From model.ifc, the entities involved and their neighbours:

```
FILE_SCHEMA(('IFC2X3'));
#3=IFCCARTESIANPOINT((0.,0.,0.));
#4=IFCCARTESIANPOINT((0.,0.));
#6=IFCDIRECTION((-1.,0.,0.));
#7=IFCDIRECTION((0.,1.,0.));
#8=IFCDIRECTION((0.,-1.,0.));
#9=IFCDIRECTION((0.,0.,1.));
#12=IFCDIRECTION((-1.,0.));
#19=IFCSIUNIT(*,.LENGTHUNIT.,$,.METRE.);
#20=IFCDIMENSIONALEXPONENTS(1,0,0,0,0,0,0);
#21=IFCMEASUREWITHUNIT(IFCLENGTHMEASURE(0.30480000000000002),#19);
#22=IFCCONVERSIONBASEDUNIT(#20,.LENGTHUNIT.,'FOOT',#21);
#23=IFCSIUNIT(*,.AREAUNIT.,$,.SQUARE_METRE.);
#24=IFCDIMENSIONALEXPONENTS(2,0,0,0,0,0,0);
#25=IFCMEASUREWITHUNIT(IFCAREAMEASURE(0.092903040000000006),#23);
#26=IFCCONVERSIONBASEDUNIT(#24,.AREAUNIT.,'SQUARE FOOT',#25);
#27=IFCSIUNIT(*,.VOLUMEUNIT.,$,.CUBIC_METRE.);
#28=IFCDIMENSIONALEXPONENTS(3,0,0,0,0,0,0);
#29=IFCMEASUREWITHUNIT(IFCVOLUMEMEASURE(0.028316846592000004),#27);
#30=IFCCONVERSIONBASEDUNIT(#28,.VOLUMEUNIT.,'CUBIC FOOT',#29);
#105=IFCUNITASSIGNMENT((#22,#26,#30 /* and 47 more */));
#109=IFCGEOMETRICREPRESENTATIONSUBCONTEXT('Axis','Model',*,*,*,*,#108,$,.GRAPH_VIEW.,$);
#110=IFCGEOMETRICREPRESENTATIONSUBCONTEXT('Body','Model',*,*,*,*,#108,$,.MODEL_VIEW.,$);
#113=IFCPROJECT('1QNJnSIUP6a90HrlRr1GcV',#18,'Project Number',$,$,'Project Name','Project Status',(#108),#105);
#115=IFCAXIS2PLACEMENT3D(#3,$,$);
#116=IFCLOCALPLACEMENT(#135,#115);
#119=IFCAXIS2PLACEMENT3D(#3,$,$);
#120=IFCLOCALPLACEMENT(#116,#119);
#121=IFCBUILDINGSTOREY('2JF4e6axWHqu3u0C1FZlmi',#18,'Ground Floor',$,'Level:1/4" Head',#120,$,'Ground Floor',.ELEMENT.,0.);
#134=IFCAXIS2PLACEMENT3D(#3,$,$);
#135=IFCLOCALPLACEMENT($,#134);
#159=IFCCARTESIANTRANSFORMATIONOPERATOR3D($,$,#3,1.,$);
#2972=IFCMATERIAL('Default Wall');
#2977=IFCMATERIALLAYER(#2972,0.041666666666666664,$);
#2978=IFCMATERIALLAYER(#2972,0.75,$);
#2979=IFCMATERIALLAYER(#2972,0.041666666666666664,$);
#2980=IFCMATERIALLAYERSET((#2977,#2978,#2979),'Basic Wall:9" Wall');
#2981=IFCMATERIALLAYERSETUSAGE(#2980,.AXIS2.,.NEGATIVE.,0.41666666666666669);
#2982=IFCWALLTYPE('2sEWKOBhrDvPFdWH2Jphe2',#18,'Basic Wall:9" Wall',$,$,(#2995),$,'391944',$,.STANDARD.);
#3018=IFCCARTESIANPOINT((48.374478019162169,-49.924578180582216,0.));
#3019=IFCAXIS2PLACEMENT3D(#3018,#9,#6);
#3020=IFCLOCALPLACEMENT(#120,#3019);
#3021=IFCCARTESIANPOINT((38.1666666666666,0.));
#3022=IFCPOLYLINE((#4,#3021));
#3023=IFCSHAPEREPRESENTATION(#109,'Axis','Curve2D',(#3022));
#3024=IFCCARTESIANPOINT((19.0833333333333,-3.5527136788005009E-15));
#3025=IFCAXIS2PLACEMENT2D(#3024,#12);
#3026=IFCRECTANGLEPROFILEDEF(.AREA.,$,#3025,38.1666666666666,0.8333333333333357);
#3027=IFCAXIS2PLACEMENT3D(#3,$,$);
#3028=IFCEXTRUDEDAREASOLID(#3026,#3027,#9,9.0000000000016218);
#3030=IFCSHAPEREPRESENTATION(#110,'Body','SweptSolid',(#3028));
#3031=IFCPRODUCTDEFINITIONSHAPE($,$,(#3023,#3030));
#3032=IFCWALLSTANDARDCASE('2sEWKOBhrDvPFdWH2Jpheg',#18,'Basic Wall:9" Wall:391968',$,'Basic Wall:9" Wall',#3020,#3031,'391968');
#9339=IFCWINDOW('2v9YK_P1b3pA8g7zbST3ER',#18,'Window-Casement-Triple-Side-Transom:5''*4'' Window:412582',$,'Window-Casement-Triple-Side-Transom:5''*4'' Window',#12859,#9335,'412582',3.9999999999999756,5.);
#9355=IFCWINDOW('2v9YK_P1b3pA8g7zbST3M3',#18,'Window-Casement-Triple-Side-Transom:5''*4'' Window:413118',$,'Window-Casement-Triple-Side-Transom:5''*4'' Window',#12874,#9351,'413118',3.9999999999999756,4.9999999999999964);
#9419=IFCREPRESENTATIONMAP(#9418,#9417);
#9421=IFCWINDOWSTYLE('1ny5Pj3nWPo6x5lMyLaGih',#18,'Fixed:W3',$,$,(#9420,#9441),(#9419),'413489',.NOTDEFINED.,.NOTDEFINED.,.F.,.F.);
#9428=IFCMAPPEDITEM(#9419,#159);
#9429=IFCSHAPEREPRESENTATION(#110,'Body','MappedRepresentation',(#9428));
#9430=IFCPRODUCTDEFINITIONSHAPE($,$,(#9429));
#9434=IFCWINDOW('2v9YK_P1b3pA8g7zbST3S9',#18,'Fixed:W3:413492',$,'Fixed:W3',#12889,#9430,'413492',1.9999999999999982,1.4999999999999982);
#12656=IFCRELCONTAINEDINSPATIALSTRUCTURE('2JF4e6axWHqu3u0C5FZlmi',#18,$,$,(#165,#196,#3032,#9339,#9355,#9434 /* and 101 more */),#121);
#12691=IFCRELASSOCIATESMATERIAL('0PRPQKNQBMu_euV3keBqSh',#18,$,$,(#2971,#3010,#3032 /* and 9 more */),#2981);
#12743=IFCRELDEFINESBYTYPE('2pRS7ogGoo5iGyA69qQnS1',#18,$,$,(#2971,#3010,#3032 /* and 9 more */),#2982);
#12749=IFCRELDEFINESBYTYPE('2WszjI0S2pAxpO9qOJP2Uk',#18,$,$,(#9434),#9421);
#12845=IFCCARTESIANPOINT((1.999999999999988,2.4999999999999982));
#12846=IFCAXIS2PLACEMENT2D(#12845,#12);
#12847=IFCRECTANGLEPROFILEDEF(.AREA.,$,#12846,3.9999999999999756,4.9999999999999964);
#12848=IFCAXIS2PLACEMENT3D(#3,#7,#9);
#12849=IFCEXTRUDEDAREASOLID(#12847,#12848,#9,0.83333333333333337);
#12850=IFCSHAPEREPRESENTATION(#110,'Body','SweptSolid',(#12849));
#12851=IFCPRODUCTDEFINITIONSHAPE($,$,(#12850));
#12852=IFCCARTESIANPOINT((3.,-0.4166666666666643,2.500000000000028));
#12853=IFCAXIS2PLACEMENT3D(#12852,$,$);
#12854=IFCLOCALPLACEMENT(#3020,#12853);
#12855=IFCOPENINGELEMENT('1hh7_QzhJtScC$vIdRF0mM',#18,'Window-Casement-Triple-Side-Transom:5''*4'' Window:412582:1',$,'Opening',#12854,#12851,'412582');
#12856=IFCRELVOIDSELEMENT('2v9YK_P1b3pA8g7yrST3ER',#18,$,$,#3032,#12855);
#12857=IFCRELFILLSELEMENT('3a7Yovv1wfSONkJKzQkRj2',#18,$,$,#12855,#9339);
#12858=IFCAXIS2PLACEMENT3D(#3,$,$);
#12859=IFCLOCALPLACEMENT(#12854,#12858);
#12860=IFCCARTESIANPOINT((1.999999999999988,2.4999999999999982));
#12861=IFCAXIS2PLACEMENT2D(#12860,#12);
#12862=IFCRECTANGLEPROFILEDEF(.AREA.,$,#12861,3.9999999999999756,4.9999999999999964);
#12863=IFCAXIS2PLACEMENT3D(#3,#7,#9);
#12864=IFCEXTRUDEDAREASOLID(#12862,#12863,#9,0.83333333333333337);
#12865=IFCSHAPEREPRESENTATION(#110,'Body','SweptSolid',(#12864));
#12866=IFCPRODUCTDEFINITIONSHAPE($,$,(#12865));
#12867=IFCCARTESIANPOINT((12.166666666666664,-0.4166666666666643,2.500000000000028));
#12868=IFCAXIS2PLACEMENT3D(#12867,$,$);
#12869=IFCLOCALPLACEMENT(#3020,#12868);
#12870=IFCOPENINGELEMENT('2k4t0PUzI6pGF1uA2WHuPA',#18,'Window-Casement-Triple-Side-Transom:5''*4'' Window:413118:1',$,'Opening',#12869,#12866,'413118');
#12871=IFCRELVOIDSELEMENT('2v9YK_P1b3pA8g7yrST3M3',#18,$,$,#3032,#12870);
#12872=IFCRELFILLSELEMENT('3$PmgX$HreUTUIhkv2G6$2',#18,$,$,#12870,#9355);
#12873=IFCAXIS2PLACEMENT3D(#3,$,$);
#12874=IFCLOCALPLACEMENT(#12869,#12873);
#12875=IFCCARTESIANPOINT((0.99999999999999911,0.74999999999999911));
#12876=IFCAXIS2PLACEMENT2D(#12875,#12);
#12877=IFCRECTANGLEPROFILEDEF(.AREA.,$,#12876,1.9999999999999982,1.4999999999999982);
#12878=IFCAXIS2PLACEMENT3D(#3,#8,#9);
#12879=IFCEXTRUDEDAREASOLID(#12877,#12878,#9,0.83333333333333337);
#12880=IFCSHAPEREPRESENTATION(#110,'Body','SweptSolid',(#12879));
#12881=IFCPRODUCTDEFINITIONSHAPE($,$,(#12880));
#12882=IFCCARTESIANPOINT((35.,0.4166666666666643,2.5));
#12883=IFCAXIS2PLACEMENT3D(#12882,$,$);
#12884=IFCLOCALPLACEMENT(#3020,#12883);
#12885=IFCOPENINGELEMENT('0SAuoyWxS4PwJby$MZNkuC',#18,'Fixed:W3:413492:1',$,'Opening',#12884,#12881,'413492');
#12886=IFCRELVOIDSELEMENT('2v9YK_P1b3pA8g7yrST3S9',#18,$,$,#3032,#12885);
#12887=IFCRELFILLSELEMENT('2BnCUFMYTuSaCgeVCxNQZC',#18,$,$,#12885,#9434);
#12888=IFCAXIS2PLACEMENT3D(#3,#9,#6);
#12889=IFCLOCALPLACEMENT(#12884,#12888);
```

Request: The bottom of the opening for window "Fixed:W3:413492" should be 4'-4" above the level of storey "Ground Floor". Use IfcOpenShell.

```python
import numpy as np
import ifcopenshell
import ifcopenshell.api.geometry
import ifcopenshell.geom
import ifcopenshell.util.element
import ifcopenshell.util.placement
import ifcopenshell.util.shape
import ifcopenshell.util.unit

model = ifcopenshell.open("model.ifc")
unit_scale = ifcopenshell.util.unit.calculate_unit_scale(model)

window = model.by_guid("2v9YK_P1b3pA8g7zbST3S9")
opening = window.FillsVoids[0].RelatingOpeningElement
storey = ifcopenshell.util.element.get_container(window, ifc_class="IfcBuildingStorey")
level = ifcopenshell.util.placement.get_local_placement(storey.ObjectPlacement)[2, 3]

# The opening's origin need not be at the sill, so measure its lowest point.
shape = ifcopenshell.geom.create_shape(ifcopenshell.geom.settings(), opening)
bottom = ifcopenshell.util.shape.get_shape_bottom_elevation(shape, shape.geometry) / unit_scale
dz = level + 52 * 0.0254 / unit_scale - bottom

shift = np.array([0.0, 0.0, dz])
# The window is placed relative to its opening, so it follows when the opening moves.
matrix = ifcopenshell.util.placement.get_local_placement(opening.ObjectPlacement)
matrix[:3, 3] += shift
ifcopenshell.api.geometry.edit_object_placement(
    model, product=opening, matrix=matrix, is_si=False, should_transform_children=True
)

print(f"moved by {dz * unit_scale:+.3f} m")

model.write("model_edited.ifc")
```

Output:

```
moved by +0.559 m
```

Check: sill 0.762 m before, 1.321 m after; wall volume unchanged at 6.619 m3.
